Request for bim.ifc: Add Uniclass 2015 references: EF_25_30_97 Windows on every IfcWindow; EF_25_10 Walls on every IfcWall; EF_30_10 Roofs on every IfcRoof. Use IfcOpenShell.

First a look at what the model holds.

```python
import ifcopenshell

model = ifcopenshell.open("bim.ifc")
print(model.schema)
print("classifications:", [c.Name for c in model.by_type("IfcClassification")])
for ifc_class in ("IfcDoor", "IfcRoof", "IfcStair", "IfcWall", "IfcWindow"):
    print(ifc_class, len(model.by_type(ifc_class)))
```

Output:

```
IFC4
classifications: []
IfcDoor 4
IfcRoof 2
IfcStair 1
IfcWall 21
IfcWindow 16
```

```python
import ifcopenshell
import ifcopenshell.api.classification

model = ifcopenshell.open("bim.ifc")

system = ifcopenshell.api.classification.add_classification(model, classification="Uniclass 2015")

codes = {
    "IfcWindow": ("EF_25_30_97", "Windows"),
    "IfcWall": ("EF_25_10", "Walls"),
    "IfcRoof": ("EF_30_10", "Roofs"),
}
for ifc_class, (code, name) in codes.items():
    products = model.by_type(ifc_class)
    ifcopenshell.api.classification.add_reference(
        model, products=products, classification=system, identification=code, name=name
    )
    print(code, len(products))

model.write("bim_rev.ifc")
```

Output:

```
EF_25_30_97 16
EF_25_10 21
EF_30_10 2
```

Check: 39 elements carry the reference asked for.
